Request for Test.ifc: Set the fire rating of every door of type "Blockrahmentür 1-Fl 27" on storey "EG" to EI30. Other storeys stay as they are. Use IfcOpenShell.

First a look at what the model holds.

```python
import ifcopenshell
import ifcopenshell.util.element

model = ifcopenshell.open("Test.ifc")
print(model.schema)
storey = next(s for s in model.by_type("IfcBuildingStorey") if s.Name == "EG")
doors = [e for e in ifcopenshell.util.element.get_decomposition(storey) if e.is_a("IfcDoor")]
seen = {}
for e in doors:
    element_type = ifcopenshell.util.element.get_type(e)
    key = (element_type.Name if element_type != e and element_type else None, ifcopenshell.util.element.get_pset(e, "Pset_DoorCommon", "FireRating"))
    seen[key] = seen.get(key, 0) + 1
for (name, value), count in sorted(seen.items(), key=str):
    print(count, "x", name, "|", value)
```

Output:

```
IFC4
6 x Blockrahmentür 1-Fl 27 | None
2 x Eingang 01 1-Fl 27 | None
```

```python
import ifcopenshell
import ifcopenshell.api.pset
import ifcopenshell.util.element

model = ifcopenshell.open("Test.ifc")

storey = next(s for s in model.by_type("IfcBuildingStorey") if s.Name == "EG")
doors = [e for e in ifcopenshell.util.element.get_decomposition(storey) if e.is_a("IfcDoor")]

count = 0
for e in doors:
    element_type = ifcopenshell.util.element.get_type(e)
    if element_type in (None, e) or element_type.Name != "Blockrahmentür 1-Fl 27":
        continue
    # add_pset returns the element's existing set when there is one.
    pset = ifcopenshell.api.pset.add_pset(model, product=e, name="Pset_DoorCommon")
    ifcopenshell.api.pset.edit_pset(model, pset=pset, properties={"FireRating": "EI30"})
    count += 1

print(count, "doors updated")

model.write("Test_v2.ifc")
```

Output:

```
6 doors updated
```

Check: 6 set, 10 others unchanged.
